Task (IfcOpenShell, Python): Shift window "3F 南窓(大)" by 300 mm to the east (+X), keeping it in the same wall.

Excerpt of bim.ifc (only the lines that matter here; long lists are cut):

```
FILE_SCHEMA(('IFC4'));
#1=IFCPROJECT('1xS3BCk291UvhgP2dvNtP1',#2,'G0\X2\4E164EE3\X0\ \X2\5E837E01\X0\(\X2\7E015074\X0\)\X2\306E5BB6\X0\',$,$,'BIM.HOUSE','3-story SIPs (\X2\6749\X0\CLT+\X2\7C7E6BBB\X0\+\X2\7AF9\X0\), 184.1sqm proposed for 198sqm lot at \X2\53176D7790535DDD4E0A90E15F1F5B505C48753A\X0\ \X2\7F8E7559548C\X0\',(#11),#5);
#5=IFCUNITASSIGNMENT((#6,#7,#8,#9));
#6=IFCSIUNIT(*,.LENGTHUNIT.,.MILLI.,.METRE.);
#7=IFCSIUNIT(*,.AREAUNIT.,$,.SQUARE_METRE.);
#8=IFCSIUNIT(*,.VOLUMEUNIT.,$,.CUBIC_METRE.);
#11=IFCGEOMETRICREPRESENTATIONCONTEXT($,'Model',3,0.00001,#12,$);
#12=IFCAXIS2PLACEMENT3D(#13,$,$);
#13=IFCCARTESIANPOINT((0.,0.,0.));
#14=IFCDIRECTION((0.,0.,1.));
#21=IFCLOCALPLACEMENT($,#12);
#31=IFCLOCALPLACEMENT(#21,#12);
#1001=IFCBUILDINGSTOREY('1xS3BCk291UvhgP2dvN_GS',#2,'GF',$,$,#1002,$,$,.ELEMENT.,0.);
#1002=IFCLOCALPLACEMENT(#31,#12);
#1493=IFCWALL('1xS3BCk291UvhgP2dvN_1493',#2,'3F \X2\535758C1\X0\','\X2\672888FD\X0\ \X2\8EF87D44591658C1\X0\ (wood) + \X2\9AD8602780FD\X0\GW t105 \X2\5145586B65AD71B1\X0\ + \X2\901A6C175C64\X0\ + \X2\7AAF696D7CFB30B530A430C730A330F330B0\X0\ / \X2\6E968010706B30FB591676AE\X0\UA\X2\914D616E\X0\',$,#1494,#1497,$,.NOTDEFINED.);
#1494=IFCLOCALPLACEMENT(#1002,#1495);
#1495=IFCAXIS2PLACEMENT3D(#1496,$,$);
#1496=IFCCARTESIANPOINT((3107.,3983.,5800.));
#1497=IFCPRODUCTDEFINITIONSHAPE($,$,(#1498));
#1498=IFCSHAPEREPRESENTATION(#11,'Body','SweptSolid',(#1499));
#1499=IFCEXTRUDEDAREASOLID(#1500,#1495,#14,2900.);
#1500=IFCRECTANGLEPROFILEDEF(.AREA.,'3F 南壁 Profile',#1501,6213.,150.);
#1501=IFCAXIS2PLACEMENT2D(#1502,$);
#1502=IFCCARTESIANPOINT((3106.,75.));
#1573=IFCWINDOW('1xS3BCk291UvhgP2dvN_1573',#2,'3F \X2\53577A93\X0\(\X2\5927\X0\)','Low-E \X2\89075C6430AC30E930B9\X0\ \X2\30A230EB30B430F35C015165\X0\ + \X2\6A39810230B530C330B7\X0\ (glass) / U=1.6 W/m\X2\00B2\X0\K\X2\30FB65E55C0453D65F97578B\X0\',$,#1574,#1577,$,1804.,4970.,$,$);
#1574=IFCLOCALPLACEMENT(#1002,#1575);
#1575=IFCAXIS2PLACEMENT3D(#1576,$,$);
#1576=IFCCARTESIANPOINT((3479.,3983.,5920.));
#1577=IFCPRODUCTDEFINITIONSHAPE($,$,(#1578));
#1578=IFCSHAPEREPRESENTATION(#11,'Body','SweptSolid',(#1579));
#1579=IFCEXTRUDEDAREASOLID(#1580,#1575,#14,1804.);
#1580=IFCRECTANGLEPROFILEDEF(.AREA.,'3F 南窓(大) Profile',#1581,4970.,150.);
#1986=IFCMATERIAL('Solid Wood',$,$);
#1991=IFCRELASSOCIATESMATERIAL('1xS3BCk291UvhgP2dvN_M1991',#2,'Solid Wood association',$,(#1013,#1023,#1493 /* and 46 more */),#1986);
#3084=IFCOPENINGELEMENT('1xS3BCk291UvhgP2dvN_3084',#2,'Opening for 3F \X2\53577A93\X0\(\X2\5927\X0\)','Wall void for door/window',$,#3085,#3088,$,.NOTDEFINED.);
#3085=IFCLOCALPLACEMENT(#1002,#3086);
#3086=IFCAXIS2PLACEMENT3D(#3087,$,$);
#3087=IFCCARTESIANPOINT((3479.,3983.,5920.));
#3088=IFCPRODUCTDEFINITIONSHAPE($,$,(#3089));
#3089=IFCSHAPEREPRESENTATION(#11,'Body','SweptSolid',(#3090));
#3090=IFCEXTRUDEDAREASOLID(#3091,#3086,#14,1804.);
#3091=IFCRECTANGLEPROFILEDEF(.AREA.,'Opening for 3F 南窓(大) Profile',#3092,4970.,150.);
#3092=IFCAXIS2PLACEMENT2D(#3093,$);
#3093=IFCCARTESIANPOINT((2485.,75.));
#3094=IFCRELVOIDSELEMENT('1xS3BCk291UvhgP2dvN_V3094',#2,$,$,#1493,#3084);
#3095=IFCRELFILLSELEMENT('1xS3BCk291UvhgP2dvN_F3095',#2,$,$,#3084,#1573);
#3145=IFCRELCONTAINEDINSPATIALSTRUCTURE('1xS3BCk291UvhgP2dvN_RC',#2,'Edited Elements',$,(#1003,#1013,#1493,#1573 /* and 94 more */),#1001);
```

```python
import ifcopenshell
import ifcopenshell.api.geometry
import ifcopenshell.util.placement
import ifcopenshell.util.unit

model = ifcopenshell.open("bim.ifc")
unit_scale = ifcopenshell.util.unit.calculate_unit_scale(model)

window = model.by_guid("1xS3BCk291UvhgP2dvN_1573")
opening = window.FillsVoids[0].RelatingOpeningElement
wall = opening.VoidsElements[0].RelatingBuildingElement

wall_matrix = ifcopenshell.util.placement.get_local_placement(wall.ObjectPlacement)
shift = wall_matrix[:3, 0] * 0.3 / unit_scale
before = ifcopenshell.util.placement.get_local_placement(window.ObjectPlacement)[:3, 3].copy()

# The window is not placed relative to its opening, so move both.
for product in (opening, window):
    matrix = ifcopenshell.util.placement.get_local_placement(product.ObjectPlacement)
    matrix[:3, 3] += shift
    ifcopenshell.api.geometry.edit_object_placement(model, product=product, matrix=matrix, is_si=False)

after = ifcopenshell.util.placement.get_local_placement(window.ObjectPlacement)[:3, 3]
print("window moved by", (after - before).round(3) + 0.0)

model.write("bim-out.ifc")
```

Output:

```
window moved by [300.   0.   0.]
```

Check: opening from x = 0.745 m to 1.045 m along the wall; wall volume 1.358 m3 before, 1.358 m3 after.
